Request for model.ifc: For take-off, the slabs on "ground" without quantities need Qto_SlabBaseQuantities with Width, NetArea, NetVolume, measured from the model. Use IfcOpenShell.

First a look at what the model holds.

```python
import ifcopenshell
import ifcopenshell.util.element
import ifcopenshell.util.unit

model = ifcopenshell.open("model.ifc")
print(model.schema)
for unit_type in ("LENGTHUNIT", "AREAUNIT", "VOLUMEUNIT"):
    print(unit_type, ifcopenshell.util.unit.calculate_unit_scale(model, unit_type))
storey = next(s for s in model.by_type("IfcBuildingStorey") if s.Name == "ground")
slabs = [e for e in ifcopenshell.util.element.get_decomposition(storey) if e.is_a("IfcSlab")]
for e in sorted(slabs, key=lambda e: e.id()):
    print(e.id(), e.is_a(), e.Name, list(ifcopenshell.util.element.get_psets(e, qtos_only=True)), sep=" | ")
```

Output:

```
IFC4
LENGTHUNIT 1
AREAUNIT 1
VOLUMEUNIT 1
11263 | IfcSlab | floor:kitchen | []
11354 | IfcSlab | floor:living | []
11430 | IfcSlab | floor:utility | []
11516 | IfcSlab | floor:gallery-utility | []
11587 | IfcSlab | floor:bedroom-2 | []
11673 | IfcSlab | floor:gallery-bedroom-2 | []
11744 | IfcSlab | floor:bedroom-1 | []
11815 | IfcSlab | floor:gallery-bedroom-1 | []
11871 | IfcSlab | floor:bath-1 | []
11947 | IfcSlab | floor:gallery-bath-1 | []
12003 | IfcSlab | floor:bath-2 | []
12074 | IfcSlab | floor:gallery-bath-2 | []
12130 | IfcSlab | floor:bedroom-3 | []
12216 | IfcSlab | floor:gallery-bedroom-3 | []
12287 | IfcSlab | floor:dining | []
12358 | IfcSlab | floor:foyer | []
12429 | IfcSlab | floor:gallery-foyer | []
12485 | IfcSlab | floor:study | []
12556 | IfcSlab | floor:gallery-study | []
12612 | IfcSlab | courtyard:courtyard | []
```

```python
import ifcopenshell
import ifcopenshell.api.pset
import ifcopenshell.geom
import ifcopenshell.util.element
import ifcopenshell.util.shape
import ifcopenshell.util.unit

model = ifcopenshell.open("model.ifc")
unit_scale = ifcopenshell.util.unit.calculate_unit_scale(model)
area_scale = ifcopenshell.util.unit.calculate_unit_scale(model, "AREAUNIT")
volume_scale = ifcopenshell.util.unit.calculate_unit_scale(model, "VOLUMEUNIT")
settings = ifcopenshell.geom.settings()

storey = next(s for s in model.by_type("IfcBuildingStorey") if s.Name == "ground")
slabs = [e for e in ifcopenshell.util.element.get_decomposition(storey) if e.is_a("IfcSlab")]

for e in sorted(slabs, key=lambda e: e.id()):
    if ifcopenshell.util.element.get_psets(e, qtos_only=True, should_inherit=False):
        continue
    # Geometry comes back in metres, in the element's own axes.
    shape = ifcopenshell.geom.create_shape(settings, e)
    values = {
        "Width": ifcopenshell.util.shape.get_z(shape.geometry) / unit_scale,
        "NetArea": ifcopenshell.util.shape.get_footprint_area(shape.geometry) / area_scale,
        "NetVolume": ifcopenshell.util.shape.get_volume(shape.geometry) / volume_scale,
    }
    qto = ifcopenshell.api.pset.add_qto(model, product=e, name="Qto_SlabBaseQuantities")
    ifcopenshell.api.pset.edit_qto(model, qto=qto, properties=values)
    print(e.id(), {k: round(v, 3) for k, v in values.items()})

model.write("model_edited.ifc")
```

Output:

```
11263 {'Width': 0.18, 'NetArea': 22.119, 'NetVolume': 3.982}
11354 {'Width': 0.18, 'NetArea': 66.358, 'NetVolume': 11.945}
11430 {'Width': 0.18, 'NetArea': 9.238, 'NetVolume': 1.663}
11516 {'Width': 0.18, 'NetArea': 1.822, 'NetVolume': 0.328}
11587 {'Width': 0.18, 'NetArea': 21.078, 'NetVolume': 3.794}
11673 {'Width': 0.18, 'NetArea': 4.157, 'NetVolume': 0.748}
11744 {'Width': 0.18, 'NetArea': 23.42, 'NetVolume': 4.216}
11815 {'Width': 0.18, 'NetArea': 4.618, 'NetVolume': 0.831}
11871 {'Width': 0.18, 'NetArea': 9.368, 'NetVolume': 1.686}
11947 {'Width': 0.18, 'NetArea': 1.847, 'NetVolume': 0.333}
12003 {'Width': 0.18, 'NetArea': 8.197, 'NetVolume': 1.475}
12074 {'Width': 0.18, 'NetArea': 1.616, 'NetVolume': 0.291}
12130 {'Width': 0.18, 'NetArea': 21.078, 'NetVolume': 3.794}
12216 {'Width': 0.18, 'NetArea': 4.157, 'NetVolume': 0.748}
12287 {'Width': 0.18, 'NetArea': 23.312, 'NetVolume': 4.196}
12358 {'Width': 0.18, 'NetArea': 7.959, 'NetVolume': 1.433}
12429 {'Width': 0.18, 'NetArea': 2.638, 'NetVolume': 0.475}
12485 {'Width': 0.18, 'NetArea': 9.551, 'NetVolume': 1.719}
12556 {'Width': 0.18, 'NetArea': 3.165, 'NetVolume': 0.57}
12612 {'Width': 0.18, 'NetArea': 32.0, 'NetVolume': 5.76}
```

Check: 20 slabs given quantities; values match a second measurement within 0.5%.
